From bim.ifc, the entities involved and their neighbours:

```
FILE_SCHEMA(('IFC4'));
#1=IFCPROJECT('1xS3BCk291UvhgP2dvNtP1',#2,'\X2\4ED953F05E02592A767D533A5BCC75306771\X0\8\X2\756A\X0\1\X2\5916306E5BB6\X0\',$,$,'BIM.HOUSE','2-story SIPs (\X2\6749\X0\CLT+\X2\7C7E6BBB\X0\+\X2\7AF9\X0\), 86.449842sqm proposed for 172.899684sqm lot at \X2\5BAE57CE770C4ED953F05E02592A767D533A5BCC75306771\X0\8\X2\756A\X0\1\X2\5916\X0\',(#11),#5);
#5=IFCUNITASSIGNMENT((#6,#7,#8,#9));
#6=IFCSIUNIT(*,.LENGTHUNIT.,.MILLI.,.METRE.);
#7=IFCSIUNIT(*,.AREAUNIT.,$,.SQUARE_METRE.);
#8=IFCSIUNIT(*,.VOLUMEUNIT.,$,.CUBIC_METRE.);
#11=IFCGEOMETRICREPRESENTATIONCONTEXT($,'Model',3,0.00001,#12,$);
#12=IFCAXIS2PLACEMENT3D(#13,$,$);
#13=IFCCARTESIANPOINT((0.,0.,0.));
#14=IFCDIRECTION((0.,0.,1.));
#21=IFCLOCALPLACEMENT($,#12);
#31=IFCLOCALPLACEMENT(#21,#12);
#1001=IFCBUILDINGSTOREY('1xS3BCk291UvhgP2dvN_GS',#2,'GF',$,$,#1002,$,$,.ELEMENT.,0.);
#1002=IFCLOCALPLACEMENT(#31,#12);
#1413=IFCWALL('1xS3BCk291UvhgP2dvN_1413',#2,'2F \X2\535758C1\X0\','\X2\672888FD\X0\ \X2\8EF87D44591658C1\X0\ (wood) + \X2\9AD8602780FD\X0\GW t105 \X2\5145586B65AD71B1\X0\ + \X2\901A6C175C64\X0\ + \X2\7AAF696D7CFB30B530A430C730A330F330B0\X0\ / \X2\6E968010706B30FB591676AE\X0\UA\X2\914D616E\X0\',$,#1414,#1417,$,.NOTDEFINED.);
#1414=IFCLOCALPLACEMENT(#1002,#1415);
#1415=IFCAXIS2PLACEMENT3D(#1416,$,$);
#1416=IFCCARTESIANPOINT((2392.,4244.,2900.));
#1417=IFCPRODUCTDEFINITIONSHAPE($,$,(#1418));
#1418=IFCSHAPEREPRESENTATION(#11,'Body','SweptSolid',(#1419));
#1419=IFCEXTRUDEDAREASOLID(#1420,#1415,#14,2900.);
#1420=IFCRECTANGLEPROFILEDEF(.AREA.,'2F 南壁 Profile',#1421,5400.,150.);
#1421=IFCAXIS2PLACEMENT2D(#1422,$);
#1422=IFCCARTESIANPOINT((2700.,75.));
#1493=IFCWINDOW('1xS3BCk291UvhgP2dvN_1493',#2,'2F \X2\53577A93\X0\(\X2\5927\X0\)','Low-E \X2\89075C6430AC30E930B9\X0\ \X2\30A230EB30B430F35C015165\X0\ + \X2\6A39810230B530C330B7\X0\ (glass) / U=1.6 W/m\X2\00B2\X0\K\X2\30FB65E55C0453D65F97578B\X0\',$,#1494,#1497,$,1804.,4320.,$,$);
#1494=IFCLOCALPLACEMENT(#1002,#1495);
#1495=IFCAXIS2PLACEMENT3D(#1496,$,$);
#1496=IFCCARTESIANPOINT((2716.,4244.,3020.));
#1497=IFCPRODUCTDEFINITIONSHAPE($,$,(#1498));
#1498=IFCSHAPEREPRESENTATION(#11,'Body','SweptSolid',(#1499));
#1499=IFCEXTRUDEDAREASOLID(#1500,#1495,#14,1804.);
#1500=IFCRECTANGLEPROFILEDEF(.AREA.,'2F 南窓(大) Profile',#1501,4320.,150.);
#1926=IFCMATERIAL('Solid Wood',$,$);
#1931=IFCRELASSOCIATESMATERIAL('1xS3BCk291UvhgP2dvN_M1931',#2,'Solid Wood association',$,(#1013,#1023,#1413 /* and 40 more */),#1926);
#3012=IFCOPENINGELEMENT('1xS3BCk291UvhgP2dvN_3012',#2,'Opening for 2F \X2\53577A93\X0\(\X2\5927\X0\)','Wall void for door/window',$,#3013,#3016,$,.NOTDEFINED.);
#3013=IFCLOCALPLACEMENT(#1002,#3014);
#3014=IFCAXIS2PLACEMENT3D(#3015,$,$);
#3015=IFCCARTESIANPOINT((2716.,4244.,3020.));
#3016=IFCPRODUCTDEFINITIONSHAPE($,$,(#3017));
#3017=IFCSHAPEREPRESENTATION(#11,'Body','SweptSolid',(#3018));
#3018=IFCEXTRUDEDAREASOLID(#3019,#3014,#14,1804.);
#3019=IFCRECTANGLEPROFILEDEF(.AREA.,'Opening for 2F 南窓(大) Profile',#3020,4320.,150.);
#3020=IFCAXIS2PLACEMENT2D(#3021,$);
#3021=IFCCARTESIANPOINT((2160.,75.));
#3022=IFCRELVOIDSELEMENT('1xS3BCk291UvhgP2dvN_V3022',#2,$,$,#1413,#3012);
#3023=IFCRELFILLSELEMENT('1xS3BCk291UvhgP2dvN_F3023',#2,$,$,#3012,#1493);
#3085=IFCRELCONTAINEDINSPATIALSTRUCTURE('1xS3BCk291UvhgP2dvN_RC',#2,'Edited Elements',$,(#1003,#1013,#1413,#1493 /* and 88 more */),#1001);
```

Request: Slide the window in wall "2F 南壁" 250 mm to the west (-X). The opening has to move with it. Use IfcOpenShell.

```python
import ifcopenshell
import ifcopenshell.api.geometry
import ifcopenshell.util.placement

model = ifcopenshell.open("bim.ifc")

window = model.by_id(1493)
opening = window.FillsVoids[0].RelatingOpeningElement
wall = opening.VoidsElements[0].RelatingBuildingElement

wall_matrix = ifcopenshell.util.placement.get_local_placement(wall.ObjectPlacement)
shift = wall_matrix[:3, 0] * -250.0
before = ifcopenshell.util.placement.get_local_placement(window.ObjectPlacement)[:3, 3].copy()

# The window is not placed relative to its opening, so move both.
for product in (opening, window):
    matrix = ifcopenshell.util.placement.get_local_placement(product.ObjectPlacement)
    matrix[:3, 3] += shift
    ifcopenshell.api.geometry.edit_object_placement(model, product=product, matrix=matrix, is_si=False)

after = ifcopenshell.util.placement.get_local_placement(window.ObjectPlacement)[:3, 3]
print("window moved by", (after - before).round(3) + 0.0)

model.write("bim_updated.ifc")
```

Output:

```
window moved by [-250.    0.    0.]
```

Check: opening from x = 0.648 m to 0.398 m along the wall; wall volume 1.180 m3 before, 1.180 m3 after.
